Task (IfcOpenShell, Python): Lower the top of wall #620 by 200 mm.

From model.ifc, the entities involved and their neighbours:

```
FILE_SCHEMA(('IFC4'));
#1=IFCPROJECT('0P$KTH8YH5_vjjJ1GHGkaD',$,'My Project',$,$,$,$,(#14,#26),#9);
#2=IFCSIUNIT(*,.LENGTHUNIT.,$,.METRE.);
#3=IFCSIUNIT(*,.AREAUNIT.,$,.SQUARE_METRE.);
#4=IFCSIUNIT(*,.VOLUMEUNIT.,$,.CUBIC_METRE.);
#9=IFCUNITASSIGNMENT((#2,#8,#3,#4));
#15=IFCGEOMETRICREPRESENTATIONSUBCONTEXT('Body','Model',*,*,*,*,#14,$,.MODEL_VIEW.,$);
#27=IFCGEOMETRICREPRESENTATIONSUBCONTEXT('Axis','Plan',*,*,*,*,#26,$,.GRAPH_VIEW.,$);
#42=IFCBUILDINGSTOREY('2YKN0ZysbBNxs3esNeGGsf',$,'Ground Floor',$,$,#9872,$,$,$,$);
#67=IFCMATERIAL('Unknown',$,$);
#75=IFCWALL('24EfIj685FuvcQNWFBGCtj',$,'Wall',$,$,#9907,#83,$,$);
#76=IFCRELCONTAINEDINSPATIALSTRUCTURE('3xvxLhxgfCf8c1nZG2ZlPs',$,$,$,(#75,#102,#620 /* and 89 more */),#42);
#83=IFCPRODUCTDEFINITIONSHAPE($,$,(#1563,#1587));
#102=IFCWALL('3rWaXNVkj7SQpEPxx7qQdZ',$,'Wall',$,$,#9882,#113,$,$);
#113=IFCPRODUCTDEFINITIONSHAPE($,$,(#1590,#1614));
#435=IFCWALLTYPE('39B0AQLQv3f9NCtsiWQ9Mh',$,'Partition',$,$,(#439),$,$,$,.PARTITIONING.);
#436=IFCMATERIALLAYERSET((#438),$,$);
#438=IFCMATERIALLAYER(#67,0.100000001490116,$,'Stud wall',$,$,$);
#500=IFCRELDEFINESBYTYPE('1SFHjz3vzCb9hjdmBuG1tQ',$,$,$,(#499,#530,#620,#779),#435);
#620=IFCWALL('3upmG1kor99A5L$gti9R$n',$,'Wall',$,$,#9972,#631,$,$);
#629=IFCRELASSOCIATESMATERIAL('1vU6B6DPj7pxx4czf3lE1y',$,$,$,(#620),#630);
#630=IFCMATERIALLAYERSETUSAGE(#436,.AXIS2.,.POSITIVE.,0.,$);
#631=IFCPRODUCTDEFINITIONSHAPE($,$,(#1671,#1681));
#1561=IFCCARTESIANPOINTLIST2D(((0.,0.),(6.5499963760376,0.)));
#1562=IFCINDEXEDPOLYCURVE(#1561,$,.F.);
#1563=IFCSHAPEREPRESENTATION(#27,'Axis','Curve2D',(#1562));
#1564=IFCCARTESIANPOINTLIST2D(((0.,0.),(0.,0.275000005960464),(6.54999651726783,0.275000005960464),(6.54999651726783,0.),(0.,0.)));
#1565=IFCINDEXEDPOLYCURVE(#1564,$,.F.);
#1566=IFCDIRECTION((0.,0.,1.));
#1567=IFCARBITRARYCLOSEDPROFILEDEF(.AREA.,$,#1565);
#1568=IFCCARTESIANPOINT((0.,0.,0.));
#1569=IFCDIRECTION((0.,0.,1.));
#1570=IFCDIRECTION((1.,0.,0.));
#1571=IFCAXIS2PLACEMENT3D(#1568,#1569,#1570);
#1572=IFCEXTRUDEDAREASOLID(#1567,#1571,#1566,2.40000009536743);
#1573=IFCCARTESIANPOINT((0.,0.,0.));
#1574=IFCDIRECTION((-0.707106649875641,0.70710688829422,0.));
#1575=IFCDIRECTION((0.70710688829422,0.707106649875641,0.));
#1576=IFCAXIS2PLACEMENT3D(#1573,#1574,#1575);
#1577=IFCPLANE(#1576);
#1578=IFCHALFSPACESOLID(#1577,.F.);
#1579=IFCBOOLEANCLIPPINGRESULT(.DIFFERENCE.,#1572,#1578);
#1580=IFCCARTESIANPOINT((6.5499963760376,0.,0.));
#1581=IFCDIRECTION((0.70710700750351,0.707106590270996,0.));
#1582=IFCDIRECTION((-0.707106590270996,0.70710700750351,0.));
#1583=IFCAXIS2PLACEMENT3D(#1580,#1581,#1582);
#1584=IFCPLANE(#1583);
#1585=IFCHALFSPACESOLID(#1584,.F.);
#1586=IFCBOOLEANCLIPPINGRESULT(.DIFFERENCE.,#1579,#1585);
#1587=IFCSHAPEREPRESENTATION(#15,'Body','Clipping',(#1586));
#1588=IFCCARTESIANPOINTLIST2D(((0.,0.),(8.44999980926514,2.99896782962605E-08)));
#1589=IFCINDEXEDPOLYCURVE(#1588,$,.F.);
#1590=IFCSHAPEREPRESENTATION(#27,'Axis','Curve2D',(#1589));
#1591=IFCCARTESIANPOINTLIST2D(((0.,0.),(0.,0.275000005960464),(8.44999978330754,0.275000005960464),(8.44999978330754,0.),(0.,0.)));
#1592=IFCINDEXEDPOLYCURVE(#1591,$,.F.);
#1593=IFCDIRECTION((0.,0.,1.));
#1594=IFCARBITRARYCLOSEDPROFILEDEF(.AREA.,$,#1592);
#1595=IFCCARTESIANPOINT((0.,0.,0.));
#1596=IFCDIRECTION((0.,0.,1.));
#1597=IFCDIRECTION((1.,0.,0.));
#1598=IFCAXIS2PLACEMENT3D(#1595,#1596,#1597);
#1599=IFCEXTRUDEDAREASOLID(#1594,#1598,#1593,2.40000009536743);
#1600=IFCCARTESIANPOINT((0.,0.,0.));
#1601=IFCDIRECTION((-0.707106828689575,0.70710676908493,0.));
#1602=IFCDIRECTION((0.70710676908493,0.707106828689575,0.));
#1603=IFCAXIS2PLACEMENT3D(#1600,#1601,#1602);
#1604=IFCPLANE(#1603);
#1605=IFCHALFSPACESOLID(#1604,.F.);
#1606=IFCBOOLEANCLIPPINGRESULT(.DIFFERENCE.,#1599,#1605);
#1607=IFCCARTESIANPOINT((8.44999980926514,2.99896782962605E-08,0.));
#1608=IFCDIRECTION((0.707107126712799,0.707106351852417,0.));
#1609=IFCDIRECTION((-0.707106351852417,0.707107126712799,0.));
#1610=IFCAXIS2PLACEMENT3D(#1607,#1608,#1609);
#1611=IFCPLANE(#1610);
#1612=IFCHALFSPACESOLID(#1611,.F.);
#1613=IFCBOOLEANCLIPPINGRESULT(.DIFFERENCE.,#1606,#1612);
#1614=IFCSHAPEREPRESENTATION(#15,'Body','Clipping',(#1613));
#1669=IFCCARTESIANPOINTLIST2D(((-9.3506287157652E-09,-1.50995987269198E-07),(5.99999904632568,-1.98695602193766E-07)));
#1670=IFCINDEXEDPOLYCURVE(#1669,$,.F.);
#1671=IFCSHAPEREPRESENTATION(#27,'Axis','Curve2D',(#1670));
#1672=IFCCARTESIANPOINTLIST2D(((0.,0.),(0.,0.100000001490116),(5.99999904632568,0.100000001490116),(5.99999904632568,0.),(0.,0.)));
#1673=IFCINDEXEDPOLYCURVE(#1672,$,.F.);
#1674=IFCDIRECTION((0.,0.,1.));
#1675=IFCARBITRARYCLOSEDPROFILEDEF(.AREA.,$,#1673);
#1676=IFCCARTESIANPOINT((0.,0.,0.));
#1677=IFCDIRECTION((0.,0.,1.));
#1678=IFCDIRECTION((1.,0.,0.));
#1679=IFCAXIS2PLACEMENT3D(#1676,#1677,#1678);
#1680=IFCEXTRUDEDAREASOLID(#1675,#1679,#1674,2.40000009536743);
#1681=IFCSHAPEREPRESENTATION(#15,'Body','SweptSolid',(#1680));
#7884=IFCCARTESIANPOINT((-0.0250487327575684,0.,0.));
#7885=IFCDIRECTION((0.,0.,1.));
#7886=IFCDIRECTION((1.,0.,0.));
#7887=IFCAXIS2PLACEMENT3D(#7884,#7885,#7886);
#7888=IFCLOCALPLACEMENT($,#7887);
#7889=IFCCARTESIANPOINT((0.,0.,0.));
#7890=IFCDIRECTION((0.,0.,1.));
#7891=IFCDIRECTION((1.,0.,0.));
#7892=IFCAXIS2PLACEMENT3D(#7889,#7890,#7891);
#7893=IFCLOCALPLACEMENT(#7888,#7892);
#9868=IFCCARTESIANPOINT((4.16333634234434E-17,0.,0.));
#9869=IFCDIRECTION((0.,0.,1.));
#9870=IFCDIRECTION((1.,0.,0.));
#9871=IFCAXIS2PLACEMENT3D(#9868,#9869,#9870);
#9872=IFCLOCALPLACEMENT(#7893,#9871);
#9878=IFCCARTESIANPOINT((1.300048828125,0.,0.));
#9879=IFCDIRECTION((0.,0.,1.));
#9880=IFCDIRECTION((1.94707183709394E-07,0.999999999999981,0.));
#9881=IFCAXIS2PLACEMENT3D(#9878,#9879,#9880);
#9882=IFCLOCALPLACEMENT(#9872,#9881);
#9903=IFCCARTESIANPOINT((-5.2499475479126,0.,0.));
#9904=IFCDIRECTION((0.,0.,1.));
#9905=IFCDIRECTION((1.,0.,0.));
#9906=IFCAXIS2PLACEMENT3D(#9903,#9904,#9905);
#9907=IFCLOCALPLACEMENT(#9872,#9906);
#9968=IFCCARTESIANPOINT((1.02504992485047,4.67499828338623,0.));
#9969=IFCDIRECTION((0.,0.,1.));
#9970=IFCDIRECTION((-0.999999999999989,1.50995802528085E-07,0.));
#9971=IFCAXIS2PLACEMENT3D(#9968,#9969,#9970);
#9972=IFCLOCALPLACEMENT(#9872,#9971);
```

```python
import ifcopenshell
import ifcopenshell.geom
import ifcopenshell.util.representation
import ifcopenshell.util.shape
import ifcopenshell.util.unit

model = ifcopenshell.open("model.ifc")
unit_scale = ifcopenshell.util.unit.calculate_unit_scale(model)
settings = ifcopenshell.geom.settings()


def volume(element):
    """Net volume in cubic metres, openings subtracted."""
    shape = ifcopenshell.geom.create_shape(settings, element)
    return ifcopenshell.util.shape.get_volume(shape.geometry)


wall = model.by_guid("3upmG1kor99A5L$gti9R$n")
before = volume(wall)

body = ifcopenshell.util.representation.get_representation(wall, "Model", "Body")
solid = body.Items[0]
old_height = solid.Depth
solid.Depth -= 0.2 / unit_scale
after = volume(wall)

print(f"height {old_height:g} -> {solid.Depth:g}, volume {before:.3f} -> {after:.3f} m3")

model.write("model_updated.ifc")
```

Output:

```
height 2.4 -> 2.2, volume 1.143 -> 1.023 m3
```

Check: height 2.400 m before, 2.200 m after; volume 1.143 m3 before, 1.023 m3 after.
